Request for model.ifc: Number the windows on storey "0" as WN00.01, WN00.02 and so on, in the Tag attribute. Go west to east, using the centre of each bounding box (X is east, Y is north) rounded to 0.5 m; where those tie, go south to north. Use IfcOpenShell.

First a look at what the model holds.

```python
import ifcopenshell
import ifcopenshell.util.element
import ifcopenshell.util.placement

model = ifcopenshell.open("model.ifc")
print(model.schema)
storey = next(s for s in model.by_type("IfcBuildingStorey") if s.Name == "0")
windows = [e for e in ifcopenshell.util.element.get_decomposition(storey) if e.is_a("IfcWindow")]
for e in sorted(windows, key=lambda e: e.id()):
    origin = ifcopenshell.util.placement.get_local_placement(e.ObjectPlacement)[:3, 3]
    print(e.id(), e.Tag, e.Name, origin.round(2) + 0.0, sep=" | ")
```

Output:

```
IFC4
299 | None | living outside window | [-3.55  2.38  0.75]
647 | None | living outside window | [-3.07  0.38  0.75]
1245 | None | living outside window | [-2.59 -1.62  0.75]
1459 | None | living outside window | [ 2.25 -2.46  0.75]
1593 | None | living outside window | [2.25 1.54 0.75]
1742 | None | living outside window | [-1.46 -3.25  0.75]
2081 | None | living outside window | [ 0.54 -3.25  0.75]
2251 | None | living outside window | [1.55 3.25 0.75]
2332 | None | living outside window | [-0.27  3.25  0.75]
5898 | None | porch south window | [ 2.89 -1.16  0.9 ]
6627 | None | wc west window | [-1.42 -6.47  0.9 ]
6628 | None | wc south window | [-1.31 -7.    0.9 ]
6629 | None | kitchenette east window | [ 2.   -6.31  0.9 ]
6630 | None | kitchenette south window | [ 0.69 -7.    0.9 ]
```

```python
import ifcopenshell
import ifcopenshell.geom
import ifcopenshell.util.element
import ifcopenshell.util.shape

model = ifcopenshell.open("model.ifc")
settings = ifcopenshell.geom.settings()
settings.set("use-world-coords", True)


def centre(element):
    shape = ifcopenshell.geom.create_shape(settings, element)
    return ifcopenshell.util.shape.get_bbox_centroid(shape.geometry)


storey = next(s for s in model.by_type("IfcBuildingStorey") if s.Name == "0")
windows = [e for e in ifcopenshell.util.element.get_decomposition(storey) if e.is_a("IfcWindow")]

# Insertion points can sit at a corner or the storey origin, so sort by the geometry (in metres).
centres = {e: centre(e) for e in windows}
windows.sort(key=lambda e: (round(centres[e][0] / 0.5), centres[e][1]))

for i, e in enumerate(windows, start=1):
    number = f"WN00.{i:02d}"
    e.Tag = number
    print(e.id(), number)

model.write("model_updated.ifc")
```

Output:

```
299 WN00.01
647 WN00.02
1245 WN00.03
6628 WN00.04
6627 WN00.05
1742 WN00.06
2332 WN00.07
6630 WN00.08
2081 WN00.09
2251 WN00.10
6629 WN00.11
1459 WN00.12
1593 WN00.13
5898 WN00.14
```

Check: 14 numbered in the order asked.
